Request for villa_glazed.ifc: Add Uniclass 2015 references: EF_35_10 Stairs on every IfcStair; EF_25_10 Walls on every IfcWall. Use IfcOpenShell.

First a look at what the model holds.

```python
import ifcopenshell

model = ifcopenshell.open("villa_glazed.ifc")
print(model.schema)
print("classifications:", [c.Name for c in model.by_type("IfcClassification")])
for ifc_class in ("IfcDoor", "IfcRoof", "IfcStair", "IfcWall", "IfcWindow"):
    print(ifc_class, len(model.by_type(ifc_class)))
```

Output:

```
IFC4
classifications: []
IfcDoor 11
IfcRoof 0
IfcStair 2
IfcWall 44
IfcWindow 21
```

```python
import ifcopenshell
import ifcopenshell.api.classification

model = ifcopenshell.open("villa_glazed.ifc")

system = ifcopenshell.api.classification.add_classification(model, classification="Uniclass 2015")

codes = {
    "IfcStair": ("EF_35_10", "Stairs"),
    "IfcWall": ("EF_25_10", "Walls"),
}
for ifc_class, (code, name) in codes.items():
    products = model.by_type(ifc_class)
    ifcopenshell.api.classification.add_reference(
        model, products=products, classification=system, identification=code, name=name
    )
    print(code, len(products))

model.write("villa_glazed_v2.ifc")
```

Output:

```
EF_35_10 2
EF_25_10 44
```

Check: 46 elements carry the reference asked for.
